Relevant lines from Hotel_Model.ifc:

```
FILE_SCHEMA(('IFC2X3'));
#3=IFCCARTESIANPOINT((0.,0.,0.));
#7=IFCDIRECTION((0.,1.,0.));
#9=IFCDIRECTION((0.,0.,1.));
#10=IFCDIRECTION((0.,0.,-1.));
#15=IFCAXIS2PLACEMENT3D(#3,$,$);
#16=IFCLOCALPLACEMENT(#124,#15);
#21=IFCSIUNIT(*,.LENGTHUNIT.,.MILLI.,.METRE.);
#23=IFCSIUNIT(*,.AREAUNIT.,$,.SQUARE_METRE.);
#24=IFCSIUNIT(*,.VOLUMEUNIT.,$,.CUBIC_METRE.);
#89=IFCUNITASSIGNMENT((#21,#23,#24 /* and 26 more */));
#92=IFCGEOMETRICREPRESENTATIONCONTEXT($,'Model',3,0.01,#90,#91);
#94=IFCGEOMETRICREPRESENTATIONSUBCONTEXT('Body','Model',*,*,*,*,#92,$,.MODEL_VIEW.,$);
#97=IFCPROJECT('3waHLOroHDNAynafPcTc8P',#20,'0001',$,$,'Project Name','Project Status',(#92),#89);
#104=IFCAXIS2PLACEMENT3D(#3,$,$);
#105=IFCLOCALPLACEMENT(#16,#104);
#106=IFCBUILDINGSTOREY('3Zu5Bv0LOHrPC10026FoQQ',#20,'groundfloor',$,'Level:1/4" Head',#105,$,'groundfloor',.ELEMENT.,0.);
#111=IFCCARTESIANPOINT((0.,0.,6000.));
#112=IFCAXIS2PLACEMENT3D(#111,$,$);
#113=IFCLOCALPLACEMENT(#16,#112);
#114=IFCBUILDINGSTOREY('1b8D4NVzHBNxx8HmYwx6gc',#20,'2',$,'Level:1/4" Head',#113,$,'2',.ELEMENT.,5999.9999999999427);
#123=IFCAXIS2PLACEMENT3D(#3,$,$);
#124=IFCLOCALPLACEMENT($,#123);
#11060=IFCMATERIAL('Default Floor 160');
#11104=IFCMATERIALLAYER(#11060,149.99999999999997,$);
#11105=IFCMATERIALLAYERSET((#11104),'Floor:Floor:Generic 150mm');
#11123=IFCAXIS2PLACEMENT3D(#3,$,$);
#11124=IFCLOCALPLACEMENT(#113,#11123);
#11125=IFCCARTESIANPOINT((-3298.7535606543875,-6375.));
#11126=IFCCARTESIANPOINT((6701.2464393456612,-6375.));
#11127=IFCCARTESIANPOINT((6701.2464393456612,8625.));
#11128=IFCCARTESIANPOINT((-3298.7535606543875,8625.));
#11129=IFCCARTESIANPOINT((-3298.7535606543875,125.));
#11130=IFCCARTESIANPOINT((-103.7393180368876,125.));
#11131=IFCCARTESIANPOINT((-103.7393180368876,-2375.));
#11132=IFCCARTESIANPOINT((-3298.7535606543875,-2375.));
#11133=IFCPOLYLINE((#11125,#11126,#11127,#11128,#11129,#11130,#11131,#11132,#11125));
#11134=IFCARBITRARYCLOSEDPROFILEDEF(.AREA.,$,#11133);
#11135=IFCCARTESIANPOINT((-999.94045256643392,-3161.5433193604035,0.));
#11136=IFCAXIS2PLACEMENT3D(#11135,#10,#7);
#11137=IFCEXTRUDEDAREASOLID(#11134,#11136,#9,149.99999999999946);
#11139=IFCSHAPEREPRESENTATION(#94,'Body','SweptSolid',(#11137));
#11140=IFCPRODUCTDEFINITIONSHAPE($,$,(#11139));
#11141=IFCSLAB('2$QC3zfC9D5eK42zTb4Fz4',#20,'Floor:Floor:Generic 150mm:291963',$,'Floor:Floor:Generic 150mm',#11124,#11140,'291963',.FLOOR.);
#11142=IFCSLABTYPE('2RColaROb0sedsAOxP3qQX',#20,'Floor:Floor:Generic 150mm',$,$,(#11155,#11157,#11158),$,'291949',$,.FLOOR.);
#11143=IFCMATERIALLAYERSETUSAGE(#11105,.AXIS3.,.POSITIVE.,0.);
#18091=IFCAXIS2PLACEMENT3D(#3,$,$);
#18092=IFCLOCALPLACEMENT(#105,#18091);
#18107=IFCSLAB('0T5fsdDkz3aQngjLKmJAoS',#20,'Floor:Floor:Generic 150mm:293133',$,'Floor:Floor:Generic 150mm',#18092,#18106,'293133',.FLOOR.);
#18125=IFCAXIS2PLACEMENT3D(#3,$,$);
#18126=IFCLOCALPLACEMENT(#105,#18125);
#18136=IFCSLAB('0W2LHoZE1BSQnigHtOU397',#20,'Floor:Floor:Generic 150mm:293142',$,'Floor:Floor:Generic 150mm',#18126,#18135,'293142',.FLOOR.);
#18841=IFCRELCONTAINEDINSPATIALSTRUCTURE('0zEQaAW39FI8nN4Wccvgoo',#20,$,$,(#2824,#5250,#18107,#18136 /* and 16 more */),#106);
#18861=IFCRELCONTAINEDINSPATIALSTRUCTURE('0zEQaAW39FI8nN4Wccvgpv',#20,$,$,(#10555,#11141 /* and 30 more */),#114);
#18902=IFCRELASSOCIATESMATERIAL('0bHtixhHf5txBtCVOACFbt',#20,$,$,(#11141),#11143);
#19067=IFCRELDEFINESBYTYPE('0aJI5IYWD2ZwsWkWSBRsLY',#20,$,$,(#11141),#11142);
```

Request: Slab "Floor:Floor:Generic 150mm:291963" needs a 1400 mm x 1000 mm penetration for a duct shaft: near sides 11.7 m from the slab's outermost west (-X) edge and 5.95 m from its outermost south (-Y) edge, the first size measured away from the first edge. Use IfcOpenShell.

```python
import numpy as np
import ifcopenshell
import ifcopenshell.api.feature
import ifcopenshell.api.geometry
import ifcopenshell.api.root
import ifcopenshell.geom
import ifcopenshell.util.placement
import ifcopenshell.util.representation
import ifcopenshell.util.shape
import ifcopenshell.util.unit

model = ifcopenshell.open("Hotel_Model.ifc")
unit_scale = ifcopenshell.util.unit.calculate_unit_scale(model)
settings = ifcopenshell.geom.settings()


def volume(element):
    """Net volume in cubic metres, openings subtracted."""
    shape = ifcopenshell.geom.create_shape(settings, element)
    return ifcopenshell.util.shape.get_volume(shape.geometry)


slab = model.by_guid("2$QC3zfC9D5eK42zTb4Fz4")
before = volume(slab)

# Extent in the slab's own axes, in metres. The edges named are its -X and -Y sides.
slab_shape = ifcopenshell.geom.create_shape(settings, slab)
vertices = ifcopenshell.util.shape.get_vertices(slab_shape.geometry)
x_min, y_min, bottom = vertices.min(axis=0)
top = vertices[:, 2].max()

opening = ifcopenshell.api.root.create_entity(model, ifc_class="IfcOpeningElement", name="Duct shaft opening")
context = ifcopenshell.util.representation.get_context(model, "Model", "Body", "MODEL_VIEW")
width, depth = 1.4, 1
outline = [(0.0, 0.0), (width, 0.0), (width, depth), (0.0, depth), (0.0, 0.0)]
# Overshoot both faces by 50 mm so the cut is clean.
shape = ifcopenshell.api.geometry.add_slab_representation(
    model, context=context, depth=top - bottom + 0.1, polyline=outline
)
ifcopenshell.api.geometry.assign_representation(model, product=opening, representation=shape)

matrix = ifcopenshell.util.placement.get_local_placement(slab.ObjectPlacement)
matrix[:, 3] = matrix @ np.append(np.array([x_min + 11.7, y_min + 5.95, bottom - 0.05]) / unit_scale, 1.0)
ifcopenshell.api.geometry.edit_object_placement(model, product=opening, matrix=matrix, is_si=False)
ifcopenshell.api.feature.add_feature(model, feature=opening, element=slab)

after = volume(slab)

print(f"slab volume {before:.3f} -> {after:.3f} m3")

model.write("Hotel_Model_updated.ifc")
```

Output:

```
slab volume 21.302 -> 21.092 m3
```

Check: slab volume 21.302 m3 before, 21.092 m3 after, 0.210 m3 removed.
